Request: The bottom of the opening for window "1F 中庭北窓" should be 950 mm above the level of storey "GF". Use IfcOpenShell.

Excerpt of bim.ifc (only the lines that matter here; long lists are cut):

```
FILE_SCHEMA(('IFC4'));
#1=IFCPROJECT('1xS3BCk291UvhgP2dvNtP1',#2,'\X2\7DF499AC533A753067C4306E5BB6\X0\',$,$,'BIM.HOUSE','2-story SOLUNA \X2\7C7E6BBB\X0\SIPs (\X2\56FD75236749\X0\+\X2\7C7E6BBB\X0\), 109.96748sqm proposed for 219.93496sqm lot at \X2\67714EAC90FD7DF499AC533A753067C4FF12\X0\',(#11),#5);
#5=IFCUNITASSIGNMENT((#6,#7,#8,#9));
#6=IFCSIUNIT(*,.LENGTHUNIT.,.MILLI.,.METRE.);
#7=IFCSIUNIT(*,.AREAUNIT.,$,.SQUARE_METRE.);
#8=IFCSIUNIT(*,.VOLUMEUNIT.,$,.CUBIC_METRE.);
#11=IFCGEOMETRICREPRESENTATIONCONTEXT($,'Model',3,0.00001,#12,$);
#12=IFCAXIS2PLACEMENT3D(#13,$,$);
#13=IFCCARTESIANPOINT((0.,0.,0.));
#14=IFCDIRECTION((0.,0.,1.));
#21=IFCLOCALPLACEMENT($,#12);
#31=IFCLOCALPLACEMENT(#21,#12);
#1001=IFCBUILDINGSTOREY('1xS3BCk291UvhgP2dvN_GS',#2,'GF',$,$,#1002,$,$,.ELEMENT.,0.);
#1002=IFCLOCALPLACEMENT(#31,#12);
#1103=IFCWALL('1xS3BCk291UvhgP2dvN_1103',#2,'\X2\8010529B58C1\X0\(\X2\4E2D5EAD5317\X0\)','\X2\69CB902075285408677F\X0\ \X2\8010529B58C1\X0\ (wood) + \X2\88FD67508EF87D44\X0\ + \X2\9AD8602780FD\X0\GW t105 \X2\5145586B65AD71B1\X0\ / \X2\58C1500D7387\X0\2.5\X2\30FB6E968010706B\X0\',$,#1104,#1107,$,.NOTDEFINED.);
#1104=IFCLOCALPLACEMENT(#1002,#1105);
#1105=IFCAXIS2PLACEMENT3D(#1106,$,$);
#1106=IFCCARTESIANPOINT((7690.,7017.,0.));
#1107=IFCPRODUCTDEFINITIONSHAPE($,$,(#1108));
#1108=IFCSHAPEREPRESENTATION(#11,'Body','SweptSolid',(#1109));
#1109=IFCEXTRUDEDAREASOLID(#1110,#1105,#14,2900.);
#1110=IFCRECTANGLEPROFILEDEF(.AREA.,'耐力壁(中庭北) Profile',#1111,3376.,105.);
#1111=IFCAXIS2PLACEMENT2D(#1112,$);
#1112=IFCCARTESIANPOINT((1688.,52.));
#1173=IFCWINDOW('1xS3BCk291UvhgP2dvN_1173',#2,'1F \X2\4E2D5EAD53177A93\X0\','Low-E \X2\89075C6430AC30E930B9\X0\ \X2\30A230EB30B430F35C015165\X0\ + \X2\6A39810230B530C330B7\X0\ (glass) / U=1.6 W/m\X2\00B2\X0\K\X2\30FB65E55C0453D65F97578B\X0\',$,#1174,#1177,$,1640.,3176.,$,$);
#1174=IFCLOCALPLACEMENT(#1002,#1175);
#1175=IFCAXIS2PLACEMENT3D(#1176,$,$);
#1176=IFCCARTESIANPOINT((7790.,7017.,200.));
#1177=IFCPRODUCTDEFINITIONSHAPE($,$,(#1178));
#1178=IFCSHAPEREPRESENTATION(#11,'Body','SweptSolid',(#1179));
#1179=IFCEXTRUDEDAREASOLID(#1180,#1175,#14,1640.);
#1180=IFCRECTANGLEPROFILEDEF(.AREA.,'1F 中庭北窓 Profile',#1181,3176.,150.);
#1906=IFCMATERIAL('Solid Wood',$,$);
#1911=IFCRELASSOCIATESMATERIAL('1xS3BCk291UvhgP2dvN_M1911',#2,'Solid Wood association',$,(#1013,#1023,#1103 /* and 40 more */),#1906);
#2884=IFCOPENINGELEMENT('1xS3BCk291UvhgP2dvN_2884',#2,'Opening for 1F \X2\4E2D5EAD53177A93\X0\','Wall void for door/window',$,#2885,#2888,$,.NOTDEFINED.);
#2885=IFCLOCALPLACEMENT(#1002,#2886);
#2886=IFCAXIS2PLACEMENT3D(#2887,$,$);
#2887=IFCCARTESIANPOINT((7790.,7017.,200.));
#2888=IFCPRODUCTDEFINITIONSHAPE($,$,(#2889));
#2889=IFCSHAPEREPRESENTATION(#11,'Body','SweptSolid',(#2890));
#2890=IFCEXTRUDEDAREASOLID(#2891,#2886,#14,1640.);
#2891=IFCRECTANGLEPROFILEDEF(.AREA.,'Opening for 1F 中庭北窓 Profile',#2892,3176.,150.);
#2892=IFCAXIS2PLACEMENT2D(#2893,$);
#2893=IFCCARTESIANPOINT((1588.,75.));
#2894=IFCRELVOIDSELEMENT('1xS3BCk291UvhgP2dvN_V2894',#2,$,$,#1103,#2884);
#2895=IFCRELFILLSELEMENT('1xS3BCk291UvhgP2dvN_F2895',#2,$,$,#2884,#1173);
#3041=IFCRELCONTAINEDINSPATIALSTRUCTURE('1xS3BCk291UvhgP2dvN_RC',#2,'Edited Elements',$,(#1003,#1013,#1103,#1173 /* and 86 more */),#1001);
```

```python
import numpy as np
import ifcopenshell
import ifcopenshell.api.geometry
import ifcopenshell.geom
import ifcopenshell.util.element
import ifcopenshell.util.placement
import ifcopenshell.util.shape
import ifcopenshell.util.unit

model = ifcopenshell.open("bim.ifc")
unit_scale = ifcopenshell.util.unit.calculate_unit_scale(model)

window = model.by_guid("1xS3BCk291UvhgP2dvN_1173")
opening = window.FillsVoids[0].RelatingOpeningElement
storey = ifcopenshell.util.element.get_container(window, ifc_class="IfcBuildingStorey")
level = ifcopenshell.util.placement.get_local_placement(storey.ObjectPlacement)[2, 3]

# The opening's origin need not be at the sill, so measure its lowest point.
shape = ifcopenshell.geom.create_shape(ifcopenshell.geom.settings(), opening)
bottom = ifcopenshell.util.shape.get_shape_bottom_elevation(shape, shape.geometry) / unit_scale
dz = level + 0.95 / unit_scale - bottom

shift = np.array([0.0, 0.0, dz])
# The window is not placed relative to its opening, so move both.
for product in (opening, window):
    matrix = ifcopenshell.util.placement.get_local_placement(product.ObjectPlacement)
    matrix[:3, 3] += shift
    ifcopenshell.api.geometry.edit_object_placement(model, product=product, matrix=matrix, is_si=False)

print(f"moved by {dz * unit_scale:+.3f} m")

model.write("bim_v2.ifc")
```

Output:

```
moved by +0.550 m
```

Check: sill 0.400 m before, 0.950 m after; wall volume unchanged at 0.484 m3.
